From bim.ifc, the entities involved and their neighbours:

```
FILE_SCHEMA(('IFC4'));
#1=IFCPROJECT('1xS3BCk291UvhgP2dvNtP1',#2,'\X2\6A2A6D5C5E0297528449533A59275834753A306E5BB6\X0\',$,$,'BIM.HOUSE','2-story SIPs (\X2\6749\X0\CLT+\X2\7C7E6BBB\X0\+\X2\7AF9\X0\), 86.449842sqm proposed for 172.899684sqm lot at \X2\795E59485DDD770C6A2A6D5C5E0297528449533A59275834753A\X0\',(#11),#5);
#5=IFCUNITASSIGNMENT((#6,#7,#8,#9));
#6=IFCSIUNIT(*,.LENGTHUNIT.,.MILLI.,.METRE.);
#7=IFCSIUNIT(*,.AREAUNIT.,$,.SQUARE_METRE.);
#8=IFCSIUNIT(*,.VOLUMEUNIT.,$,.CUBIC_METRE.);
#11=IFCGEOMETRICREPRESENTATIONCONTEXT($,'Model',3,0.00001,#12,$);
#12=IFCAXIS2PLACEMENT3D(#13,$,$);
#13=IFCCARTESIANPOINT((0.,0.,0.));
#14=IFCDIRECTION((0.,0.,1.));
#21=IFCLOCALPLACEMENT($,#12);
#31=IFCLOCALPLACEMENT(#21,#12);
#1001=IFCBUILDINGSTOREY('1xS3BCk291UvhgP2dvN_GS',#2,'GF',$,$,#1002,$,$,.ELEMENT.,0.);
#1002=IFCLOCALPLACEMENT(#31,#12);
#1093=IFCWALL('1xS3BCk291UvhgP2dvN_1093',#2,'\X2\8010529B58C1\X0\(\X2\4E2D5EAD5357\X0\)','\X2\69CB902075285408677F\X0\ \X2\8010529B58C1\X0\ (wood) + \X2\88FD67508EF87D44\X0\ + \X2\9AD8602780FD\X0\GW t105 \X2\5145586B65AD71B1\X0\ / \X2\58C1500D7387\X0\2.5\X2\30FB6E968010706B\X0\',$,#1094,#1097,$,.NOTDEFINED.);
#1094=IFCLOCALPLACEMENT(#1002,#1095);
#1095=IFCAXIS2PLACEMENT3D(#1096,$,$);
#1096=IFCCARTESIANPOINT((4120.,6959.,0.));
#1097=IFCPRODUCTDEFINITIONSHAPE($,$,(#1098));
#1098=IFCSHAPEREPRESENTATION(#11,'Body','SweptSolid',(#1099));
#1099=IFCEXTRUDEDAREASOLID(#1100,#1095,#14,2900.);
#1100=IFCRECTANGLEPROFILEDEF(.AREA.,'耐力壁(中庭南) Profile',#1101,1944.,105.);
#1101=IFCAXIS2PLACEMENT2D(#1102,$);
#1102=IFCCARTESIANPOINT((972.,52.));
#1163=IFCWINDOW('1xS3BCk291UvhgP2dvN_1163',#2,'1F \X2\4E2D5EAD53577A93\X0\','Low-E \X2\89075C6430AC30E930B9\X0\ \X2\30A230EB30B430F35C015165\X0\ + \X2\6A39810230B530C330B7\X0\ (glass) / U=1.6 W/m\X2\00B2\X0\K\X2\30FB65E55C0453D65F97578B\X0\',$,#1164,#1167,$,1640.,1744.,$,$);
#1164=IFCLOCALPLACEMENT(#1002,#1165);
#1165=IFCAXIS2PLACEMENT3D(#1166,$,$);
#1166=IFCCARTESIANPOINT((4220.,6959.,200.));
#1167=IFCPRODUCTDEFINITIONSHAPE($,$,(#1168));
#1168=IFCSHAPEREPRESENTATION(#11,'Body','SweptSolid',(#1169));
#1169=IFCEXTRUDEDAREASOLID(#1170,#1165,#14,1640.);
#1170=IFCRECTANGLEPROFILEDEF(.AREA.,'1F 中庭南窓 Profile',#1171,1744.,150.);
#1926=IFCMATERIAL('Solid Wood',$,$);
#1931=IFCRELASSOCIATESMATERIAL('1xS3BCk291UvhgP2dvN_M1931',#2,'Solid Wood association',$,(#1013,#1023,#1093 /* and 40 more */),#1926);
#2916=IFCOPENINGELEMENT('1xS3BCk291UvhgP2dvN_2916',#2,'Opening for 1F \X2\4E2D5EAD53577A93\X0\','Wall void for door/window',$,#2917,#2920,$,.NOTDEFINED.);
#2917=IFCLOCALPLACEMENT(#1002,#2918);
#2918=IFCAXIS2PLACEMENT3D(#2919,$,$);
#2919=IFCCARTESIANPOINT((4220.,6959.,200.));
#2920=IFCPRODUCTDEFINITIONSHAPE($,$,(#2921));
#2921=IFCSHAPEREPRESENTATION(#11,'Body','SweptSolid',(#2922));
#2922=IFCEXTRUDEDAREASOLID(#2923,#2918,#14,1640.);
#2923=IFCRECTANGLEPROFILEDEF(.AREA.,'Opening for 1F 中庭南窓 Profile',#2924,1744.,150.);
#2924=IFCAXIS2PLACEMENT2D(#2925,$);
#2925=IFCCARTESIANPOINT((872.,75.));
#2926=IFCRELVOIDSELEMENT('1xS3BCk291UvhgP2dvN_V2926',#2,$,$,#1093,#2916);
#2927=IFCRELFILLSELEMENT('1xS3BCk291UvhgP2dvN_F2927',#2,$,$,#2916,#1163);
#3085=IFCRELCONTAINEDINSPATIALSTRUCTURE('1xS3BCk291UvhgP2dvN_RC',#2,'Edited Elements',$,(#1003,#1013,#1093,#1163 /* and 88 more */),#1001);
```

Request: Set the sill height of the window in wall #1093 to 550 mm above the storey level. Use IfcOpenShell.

```python
import numpy as np
import ifcopenshell
import ifcopenshell.api.geometry
import ifcopenshell.geom
import ifcopenshell.util.element
import ifcopenshell.util.placement
import ifcopenshell.util.shape
import ifcopenshell.util.unit

model = ifcopenshell.open("bim.ifc")
unit_scale = ifcopenshell.util.unit.calculate_unit_scale(model)

window = model.by_id(1163)
opening = window.FillsVoids[0].RelatingOpeningElement
storey = ifcopenshell.util.element.get_container(window, ifc_class="IfcBuildingStorey")
level = ifcopenshell.util.placement.get_local_placement(storey.ObjectPlacement)[2, 3]

# The opening's origin need not be at the sill, so measure its lowest point.
shape = ifcopenshell.geom.create_shape(ifcopenshell.geom.settings(), opening)
bottom = ifcopenshell.util.shape.get_shape_bottom_elevation(shape, shape.geometry) / unit_scale
dz = level + 0.55 / unit_scale - bottom

shift = np.array([0.0, 0.0, dz])
# The window is not placed relative to its opening, so move both.
for product in (opening, window):
    matrix = ifcopenshell.util.placement.get_local_placement(product.ObjectPlacement)
    matrix[:3, 3] += shift
    ifcopenshell.api.geometry.edit_object_placement(model, product=product, matrix=matrix, is_si=False)

print(f"moved by {dz * unit_scale:+.3f} m")

model.write("bim_updated.ifc")
```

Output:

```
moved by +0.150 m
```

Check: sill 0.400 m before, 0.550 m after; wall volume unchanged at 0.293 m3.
